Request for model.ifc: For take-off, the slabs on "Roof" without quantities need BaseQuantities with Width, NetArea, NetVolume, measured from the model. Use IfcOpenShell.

First a look at what the model holds.

```python
import ifcopenshell
import ifcopenshell.util.element
import ifcopenshell.util.unit

model = ifcopenshell.open("model.ifc")
print(model.schema)
for unit_type in ("LENGTHUNIT", "AREAUNIT", "VOLUMEUNIT"):
    print(unit_type, ifcopenshell.util.unit.calculate_unit_scale(model, unit_type))
storey = next(s for s in model.by_type("IfcBuildingStorey") if s.Name == "Roof")
slabs = [e for e in ifcopenshell.util.element.get_decomposition(storey) if e.is_a("IfcSlab")]
for e in sorted(slabs, key=lambda e: e.id()):
    print(e.id(), e.is_a(), e.Name, list(ifcopenshell.util.element.get_psets(e, qtos_only=True)), sep=" | ")
```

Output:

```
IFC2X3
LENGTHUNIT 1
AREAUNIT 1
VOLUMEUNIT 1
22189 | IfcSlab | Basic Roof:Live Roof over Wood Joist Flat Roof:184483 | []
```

```python
import ifcopenshell
import ifcopenshell.api.pset
import ifcopenshell.geom
import ifcopenshell.util.element
import ifcopenshell.util.shape
import ifcopenshell.util.unit

model = ifcopenshell.open("model.ifc")
unit_scale = ifcopenshell.util.unit.calculate_unit_scale(model)
area_scale = ifcopenshell.util.unit.calculate_unit_scale(model, "AREAUNIT")
volume_scale = ifcopenshell.util.unit.calculate_unit_scale(model, "VOLUMEUNIT")
settings = ifcopenshell.geom.settings()

storey = next(s for s in model.by_type("IfcBuildingStorey") if s.Name == "Roof")
slabs = [e for e in ifcopenshell.util.element.get_decomposition(storey) if e.is_a("IfcSlab")]

for e in sorted(slabs, key=lambda e: e.id()):
    if ifcopenshell.util.element.get_psets(e, qtos_only=True, should_inherit=False):
        continue
    # Geometry comes back in metres, in the element's own axes.
    shape = ifcopenshell.geom.create_shape(settings, e)
    values = {
        "Width": ifcopenshell.util.shape.get_z(shape.geometry) / unit_scale,
        "NetArea": ifcopenshell.util.shape.get_footprint_area(shape.geometry) / area_scale,
        "NetVolume": ifcopenshell.util.shape.get_volume(shape.geometry) / volume_scale,
    }
    qto = ifcopenshell.api.pset.add_qto(model, product=e, name="BaseQuantities")
    ifcopenshell.api.pset.edit_qto(model, qto=qto, properties=values)
    print(e.id(), {k: round(v, 3) for k, v in values.items()})

model.write("model-out.ifc")
```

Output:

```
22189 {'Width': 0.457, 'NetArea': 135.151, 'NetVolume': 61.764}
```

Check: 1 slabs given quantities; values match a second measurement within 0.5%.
